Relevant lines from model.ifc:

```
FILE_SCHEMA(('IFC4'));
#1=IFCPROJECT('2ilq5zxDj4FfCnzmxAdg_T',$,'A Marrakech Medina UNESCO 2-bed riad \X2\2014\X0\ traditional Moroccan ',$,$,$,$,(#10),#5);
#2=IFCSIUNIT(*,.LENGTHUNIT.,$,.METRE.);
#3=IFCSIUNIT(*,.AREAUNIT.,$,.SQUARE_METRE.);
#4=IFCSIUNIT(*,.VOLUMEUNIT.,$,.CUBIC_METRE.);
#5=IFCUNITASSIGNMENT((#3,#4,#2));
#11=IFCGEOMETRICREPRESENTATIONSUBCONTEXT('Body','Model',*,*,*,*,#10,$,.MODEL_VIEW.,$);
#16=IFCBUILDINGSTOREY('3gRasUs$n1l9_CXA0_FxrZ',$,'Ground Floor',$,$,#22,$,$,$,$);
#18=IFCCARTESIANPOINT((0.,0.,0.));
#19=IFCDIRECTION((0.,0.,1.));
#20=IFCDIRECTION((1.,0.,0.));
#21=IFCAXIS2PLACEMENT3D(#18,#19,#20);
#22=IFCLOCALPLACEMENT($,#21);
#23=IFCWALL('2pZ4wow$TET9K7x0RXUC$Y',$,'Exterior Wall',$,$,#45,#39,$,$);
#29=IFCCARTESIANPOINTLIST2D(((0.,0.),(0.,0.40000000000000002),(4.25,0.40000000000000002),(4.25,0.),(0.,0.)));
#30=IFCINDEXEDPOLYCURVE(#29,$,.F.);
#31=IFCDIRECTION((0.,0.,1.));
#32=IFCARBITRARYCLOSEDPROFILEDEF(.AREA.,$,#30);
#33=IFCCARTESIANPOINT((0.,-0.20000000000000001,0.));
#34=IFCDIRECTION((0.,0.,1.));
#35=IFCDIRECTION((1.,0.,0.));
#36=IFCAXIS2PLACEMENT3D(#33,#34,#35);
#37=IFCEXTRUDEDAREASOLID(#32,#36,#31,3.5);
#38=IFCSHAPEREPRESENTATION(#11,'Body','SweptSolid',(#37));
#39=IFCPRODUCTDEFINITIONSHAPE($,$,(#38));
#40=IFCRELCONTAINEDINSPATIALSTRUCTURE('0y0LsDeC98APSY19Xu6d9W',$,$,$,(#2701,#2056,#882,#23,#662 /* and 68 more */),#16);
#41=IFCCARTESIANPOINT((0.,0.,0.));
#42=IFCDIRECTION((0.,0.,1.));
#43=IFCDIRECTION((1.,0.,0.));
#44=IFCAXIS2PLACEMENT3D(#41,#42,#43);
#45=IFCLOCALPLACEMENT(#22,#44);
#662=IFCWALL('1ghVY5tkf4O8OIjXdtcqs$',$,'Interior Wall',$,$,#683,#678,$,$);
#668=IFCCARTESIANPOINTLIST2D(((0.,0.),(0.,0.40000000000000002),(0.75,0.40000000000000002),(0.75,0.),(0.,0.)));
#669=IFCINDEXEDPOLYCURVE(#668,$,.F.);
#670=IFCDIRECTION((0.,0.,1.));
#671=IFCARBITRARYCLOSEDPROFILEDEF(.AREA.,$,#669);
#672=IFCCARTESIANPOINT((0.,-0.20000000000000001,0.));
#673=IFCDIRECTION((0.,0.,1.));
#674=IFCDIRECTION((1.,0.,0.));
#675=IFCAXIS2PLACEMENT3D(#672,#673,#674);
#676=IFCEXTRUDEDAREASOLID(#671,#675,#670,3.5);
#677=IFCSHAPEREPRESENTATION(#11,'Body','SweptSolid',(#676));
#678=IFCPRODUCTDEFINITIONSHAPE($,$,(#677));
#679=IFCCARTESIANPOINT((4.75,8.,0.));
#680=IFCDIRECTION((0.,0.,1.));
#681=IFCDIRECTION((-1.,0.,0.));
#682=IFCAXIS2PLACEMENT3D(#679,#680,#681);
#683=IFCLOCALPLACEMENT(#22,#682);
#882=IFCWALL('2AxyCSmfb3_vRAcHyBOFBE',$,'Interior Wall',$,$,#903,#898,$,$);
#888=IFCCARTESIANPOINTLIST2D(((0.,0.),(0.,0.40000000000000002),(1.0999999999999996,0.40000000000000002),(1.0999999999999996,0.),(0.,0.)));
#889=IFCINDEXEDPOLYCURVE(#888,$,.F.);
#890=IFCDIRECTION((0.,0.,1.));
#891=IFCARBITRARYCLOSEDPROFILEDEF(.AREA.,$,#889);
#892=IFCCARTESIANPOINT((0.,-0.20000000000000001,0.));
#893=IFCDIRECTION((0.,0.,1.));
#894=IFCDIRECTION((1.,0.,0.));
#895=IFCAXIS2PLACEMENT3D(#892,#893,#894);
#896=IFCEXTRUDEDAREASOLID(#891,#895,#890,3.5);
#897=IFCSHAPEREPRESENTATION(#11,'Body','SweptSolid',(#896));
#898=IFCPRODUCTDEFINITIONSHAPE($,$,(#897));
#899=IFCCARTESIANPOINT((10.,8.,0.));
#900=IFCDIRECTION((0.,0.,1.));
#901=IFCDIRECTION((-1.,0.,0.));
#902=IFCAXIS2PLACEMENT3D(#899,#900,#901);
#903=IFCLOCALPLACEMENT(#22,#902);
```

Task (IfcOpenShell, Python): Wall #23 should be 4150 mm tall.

```python
import ifcopenshell
import ifcopenshell.geom
import ifcopenshell.util.representation
import ifcopenshell.util.shape
import ifcopenshell.util.unit

model = ifcopenshell.open("model.ifc")
unit_scale = ifcopenshell.util.unit.calculate_unit_scale(model)
settings = ifcopenshell.geom.settings()


def volume(element):
    """Net volume in cubic metres, openings subtracted."""
    shape = ifcopenshell.geom.create_shape(settings, element)
    return ifcopenshell.util.shape.get_volume(shape.geometry)


wall = model.by_guid("2pZ4wow$TET9K7x0RXUC$Y")
before = volume(wall)

body = ifcopenshell.util.representation.get_representation(wall, "Model", "Body")
solid = body.Items[0]
old_height = solid.Depth
solid.Depth = 4.15 / unit_scale
after = volume(wall)

print(f"height {old_height:g} -> {solid.Depth:g}, volume {before:.3f} -> {after:.3f} m3")

model.write("model-out.ifc")
```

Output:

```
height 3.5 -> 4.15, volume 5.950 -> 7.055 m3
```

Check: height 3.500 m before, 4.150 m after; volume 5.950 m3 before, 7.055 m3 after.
